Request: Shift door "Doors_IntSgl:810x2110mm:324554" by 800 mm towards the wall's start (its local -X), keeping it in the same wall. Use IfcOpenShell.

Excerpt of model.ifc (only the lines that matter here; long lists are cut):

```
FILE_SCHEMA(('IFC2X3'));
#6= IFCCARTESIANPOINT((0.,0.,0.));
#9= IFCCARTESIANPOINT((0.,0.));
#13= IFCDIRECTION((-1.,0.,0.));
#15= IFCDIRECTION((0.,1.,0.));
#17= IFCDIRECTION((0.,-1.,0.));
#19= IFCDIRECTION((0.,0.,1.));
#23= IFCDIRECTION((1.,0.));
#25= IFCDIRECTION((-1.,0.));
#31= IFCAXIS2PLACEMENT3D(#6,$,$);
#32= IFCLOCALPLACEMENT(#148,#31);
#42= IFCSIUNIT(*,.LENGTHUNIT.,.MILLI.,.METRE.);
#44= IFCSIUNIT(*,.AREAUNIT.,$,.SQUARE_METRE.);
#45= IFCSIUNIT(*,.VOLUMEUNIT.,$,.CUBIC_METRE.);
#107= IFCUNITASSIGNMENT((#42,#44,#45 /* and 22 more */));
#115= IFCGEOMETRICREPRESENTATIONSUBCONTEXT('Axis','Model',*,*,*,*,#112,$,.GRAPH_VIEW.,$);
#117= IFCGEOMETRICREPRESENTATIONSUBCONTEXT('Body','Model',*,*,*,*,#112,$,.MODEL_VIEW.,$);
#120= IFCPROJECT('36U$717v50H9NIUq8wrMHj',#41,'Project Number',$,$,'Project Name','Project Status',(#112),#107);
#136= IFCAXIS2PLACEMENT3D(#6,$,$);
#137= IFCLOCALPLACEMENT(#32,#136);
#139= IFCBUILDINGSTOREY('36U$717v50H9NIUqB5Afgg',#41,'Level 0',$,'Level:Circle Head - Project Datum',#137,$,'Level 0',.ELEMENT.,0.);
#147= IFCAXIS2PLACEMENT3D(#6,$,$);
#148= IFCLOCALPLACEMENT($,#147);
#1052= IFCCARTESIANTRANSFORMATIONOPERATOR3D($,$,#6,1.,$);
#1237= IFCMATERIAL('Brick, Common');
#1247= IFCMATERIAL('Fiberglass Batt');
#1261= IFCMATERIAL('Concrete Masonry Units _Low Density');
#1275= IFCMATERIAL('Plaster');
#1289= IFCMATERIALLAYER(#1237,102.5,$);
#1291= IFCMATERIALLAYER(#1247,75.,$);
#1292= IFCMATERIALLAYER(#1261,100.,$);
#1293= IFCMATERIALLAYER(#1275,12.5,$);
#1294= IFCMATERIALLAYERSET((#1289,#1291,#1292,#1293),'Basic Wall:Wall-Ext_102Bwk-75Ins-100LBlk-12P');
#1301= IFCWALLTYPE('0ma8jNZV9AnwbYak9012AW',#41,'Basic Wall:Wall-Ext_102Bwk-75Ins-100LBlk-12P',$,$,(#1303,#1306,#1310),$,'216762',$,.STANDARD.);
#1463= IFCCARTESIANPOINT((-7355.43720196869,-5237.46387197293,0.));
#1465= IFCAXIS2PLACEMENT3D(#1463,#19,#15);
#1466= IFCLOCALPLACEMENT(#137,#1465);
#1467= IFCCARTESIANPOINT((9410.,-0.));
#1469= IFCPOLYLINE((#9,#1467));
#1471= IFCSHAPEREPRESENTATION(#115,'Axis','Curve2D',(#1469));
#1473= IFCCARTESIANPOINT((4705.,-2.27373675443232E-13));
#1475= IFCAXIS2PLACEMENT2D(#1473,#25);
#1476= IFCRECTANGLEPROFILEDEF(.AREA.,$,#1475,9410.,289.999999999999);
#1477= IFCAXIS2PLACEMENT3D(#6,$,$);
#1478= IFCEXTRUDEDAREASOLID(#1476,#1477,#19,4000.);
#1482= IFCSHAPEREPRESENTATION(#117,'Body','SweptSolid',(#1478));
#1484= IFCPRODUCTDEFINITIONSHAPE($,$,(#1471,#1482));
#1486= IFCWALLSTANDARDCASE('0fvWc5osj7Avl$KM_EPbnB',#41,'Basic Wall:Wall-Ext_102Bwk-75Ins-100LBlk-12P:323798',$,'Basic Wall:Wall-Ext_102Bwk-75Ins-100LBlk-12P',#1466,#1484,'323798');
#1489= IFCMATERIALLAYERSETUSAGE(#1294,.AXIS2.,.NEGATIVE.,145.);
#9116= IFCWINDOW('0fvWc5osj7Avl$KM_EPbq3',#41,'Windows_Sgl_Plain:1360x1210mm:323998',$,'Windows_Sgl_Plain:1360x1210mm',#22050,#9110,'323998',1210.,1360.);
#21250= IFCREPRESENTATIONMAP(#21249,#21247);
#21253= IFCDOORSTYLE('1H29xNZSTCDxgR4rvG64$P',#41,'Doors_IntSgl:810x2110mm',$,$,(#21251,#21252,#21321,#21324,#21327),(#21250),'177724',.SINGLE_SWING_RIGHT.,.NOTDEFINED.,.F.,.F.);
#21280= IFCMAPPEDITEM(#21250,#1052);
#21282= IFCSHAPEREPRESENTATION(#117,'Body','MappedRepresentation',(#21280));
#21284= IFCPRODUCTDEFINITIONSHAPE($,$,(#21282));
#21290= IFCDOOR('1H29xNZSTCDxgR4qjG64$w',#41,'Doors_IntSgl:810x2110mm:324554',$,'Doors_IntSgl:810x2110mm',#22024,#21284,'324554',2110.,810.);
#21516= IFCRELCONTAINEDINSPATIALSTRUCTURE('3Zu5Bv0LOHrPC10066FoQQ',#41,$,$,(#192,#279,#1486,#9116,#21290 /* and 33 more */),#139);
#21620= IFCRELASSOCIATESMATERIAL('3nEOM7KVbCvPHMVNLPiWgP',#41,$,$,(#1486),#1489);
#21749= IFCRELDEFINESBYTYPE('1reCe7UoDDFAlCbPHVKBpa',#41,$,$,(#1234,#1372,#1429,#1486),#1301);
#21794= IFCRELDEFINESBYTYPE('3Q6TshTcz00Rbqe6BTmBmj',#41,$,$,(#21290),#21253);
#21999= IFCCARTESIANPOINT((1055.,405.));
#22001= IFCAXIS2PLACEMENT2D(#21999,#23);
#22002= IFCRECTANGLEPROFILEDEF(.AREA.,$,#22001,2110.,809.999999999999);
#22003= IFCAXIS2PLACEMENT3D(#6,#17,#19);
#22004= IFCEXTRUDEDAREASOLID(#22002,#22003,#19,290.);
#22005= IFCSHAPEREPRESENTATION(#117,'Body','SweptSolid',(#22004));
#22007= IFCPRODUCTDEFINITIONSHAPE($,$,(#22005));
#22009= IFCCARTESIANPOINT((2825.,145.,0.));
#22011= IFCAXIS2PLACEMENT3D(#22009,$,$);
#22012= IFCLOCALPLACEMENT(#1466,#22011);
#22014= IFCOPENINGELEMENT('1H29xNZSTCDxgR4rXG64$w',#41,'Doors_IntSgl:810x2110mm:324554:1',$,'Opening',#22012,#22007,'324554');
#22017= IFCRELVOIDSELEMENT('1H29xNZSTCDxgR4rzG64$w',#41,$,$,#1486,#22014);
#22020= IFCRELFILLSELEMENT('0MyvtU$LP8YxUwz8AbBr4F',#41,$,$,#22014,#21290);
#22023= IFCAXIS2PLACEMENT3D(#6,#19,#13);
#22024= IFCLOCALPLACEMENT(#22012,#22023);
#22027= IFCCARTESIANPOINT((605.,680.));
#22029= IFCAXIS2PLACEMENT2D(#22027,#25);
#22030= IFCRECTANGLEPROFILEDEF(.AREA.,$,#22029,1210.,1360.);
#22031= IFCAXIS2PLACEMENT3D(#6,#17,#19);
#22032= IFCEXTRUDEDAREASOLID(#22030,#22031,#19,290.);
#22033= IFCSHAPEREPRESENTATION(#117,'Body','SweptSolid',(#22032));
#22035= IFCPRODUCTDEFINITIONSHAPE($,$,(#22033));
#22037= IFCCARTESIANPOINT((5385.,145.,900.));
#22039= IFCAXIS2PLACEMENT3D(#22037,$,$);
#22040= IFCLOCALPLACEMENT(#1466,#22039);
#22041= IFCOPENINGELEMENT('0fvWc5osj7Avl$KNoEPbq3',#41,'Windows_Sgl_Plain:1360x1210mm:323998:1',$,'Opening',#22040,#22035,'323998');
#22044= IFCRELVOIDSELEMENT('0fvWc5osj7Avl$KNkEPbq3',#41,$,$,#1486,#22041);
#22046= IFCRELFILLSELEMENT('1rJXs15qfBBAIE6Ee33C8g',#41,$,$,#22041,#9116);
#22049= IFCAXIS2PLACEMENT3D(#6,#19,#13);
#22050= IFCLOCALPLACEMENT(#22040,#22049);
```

```python
import ifcopenshell
import ifcopenshell.api.geometry
import ifcopenshell.util.placement
import ifcopenshell.util.unit

model = ifcopenshell.open("model.ifc")
unit_scale = ifcopenshell.util.unit.calculate_unit_scale(model)

door = model.by_guid("1H29xNZSTCDxgR4qjG64$w")
opening = door.FillsVoids[0].RelatingOpeningElement
wall = opening.VoidsElements[0].RelatingBuildingElement

wall_matrix = ifcopenshell.util.placement.get_local_placement(wall.ObjectPlacement)
shift = wall_matrix[:3, 0] * -0.8 / unit_scale
before = ifcopenshell.util.placement.get_local_placement(door.ObjectPlacement)[:3, 3].copy()

# The door is placed relative to its opening, so it follows when the opening moves.
matrix = ifcopenshell.util.placement.get_local_placement(opening.ObjectPlacement)
matrix[:3, 3] += shift
ifcopenshell.api.geometry.edit_object_placement(
    model, product=opening, matrix=matrix, is_si=False, should_transform_children=True
)

after = ifcopenshell.util.placement.get_local_placement(door.ObjectPlacement)[:3, 3]
print("door moved by", (after - before).round(3) + 0.0)

model.write("model_updated.ifc")
```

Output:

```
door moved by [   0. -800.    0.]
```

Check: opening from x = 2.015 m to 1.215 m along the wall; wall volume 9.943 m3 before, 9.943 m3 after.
